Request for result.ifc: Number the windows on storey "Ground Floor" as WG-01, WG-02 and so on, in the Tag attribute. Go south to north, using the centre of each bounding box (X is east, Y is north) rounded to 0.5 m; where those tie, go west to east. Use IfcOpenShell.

First a look at what the model holds.

```python
import ifcopenshell
import ifcopenshell.util.element
import ifcopenshell.util.placement

model = ifcopenshell.open("result.ifc")
print(model.schema)
storey = next(s for s in model.by_type("IfcBuildingStorey") if s.Name == "Ground Floor")
windows = [e for e in ifcopenshell.util.element.get_decomposition(storey) if e.is_a("IfcWindow")]
for e in sorted(windows, key=lambda e: e.id()):
    origin = ifcopenshell.util.placement.get_local_placement(e.ObjectPlacement)[:3, 3]
    print(e.id(), e.Tag, e.Name, origin.round(2) + 0.0, sep=" | ")
```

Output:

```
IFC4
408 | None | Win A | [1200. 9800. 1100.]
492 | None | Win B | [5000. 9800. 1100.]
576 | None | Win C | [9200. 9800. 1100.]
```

```python
import ifcopenshell
import ifcopenshell.geom
import ifcopenshell.util.element
import ifcopenshell.util.shape

model = ifcopenshell.open("result.ifc")
settings = ifcopenshell.geom.settings()
settings.set("use-world-coords", True)


def centre(element):
    shape = ifcopenshell.geom.create_shape(settings, element)
    return ifcopenshell.util.shape.get_bbox_centroid(shape.geometry)


storey = next(s for s in model.by_type("IfcBuildingStorey") if s.Name == "Ground Floor")
windows = [e for e in ifcopenshell.util.element.get_decomposition(storey) if e.is_a("IfcWindow")]

# Insertion points can sit at a corner or the storey origin, so sort by the geometry (in metres).
centres = {e: centre(e) for e in windows}
windows.sort(key=lambda e: (round(centres[e][1] / 0.5), centres[e][0]))

for i, e in enumerate(windows, start=1):
    number = f"WG-{i:02d}"
    e.Tag = number
    print(e.id(), number)

model.write("result-out.ifc")
```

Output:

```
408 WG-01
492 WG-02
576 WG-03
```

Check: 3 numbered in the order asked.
